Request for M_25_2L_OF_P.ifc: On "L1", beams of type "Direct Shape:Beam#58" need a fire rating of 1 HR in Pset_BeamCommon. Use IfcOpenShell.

First a look at what the model holds.

```python
import ifcopenshell
import ifcopenshell.util.element

model = ifcopenshell.open("M_25_2L_OF_P.ifc")
print(model.schema)
storey = next(s for s in model.by_type("IfcBuildingStorey") if s.Name == "L1")
beams = [e for e in ifcopenshell.util.element.get_decomposition(storey) if e.is_a("IfcBeam")]
seen = {}
for e in beams:
    element_type = ifcopenshell.util.element.get_type(e)
    key = (element_type.Name if element_type != e and element_type else None, ifcopenshell.util.element.get_pset(e, "Pset_BeamCommon", "FireRating"))
    seen[key] = seen.get(key, 0) + 1
for (name, value), count in sorted(seen.items(), key=str):
    print(count, "x", name, "|", value)
```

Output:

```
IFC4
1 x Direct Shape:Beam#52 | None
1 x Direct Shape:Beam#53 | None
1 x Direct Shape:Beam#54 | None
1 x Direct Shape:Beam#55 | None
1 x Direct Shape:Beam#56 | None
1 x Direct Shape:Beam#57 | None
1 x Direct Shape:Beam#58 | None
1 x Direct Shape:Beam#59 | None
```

```python
import ifcopenshell
import ifcopenshell.api.pset
import ifcopenshell.util.element

model = ifcopenshell.open("M_25_2L_OF_P.ifc")

storey = next(s for s in model.by_type("IfcBuildingStorey") if s.Name == "L1")
beams = [e for e in ifcopenshell.util.element.get_decomposition(storey) if e.is_a("IfcBeam")]

count = 0
for e in beams:
    element_type = ifcopenshell.util.element.get_type(e)
    if element_type in (None, e) or element_type.Name != "Direct Shape:Beam#58":
        continue
    # add_pset returns the element's existing set when there is one.
    pset = ifcopenshell.api.pset.add_pset(model, product=e, name="Pset_BeamCommon")
    ifcopenshell.api.pset.edit_pset(model, pset=pset, properties={"FireRating": "1 HR"})
    count += 1

print(count, "beams updated")

model.write("M_25_2L_OF_P_rev.ifc")
```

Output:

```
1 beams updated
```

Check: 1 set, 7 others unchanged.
